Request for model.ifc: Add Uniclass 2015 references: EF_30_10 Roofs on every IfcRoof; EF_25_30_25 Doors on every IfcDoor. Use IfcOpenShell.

First a look at what the model holds.

```python
import ifcopenshell

model = ifcopenshell.open("model.ifc")
print(model.schema)
print("classifications:", [c.Name for c in model.by_type("IfcClassification")])
for ifc_class in ("IfcDoor", "IfcRoof", "IfcStair", "IfcWall", "IfcWindow"):
    print(ifc_class, len(model.by_type(ifc_class)))
```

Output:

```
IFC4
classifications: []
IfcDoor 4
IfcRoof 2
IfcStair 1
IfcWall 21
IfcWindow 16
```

```python
import ifcopenshell
import ifcopenshell.api.classification

model = ifcopenshell.open("model.ifc")

system = ifcopenshell.api.classification.add_classification(model, classification="Uniclass 2015")

codes = {
    "IfcRoof": ("EF_30_10", "Roofs"),
    "IfcDoor": ("EF_25_30_25", "Doors"),
}
for ifc_class, (code, name) in codes.items():
    products = model.by_type(ifc_class)
    ifcopenshell.api.classification.add_reference(
        model, products=products, classification=system, identification=code, name=name
    )
    print(code, len(products))

model.write("model_edited.ifc")
```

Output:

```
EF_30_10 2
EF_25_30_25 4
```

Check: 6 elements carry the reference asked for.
